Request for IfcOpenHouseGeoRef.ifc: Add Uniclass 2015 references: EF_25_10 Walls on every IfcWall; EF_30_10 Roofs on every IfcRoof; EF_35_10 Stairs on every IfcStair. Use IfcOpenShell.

First a look at what the model holds.

```python
import ifcopenshell

model = ifcopenshell.open("IfcOpenHouseGeoRef.ifc")
print(model.schema)
print("classifications:", [c.Name for c in model.by_type("IfcClassification")])
for ifc_class in ("IfcDoor", "IfcRoof", "IfcStair", "IfcWall", "IfcWindow"):
    print(ifc_class, len(model.by_type(ifc_class)))
```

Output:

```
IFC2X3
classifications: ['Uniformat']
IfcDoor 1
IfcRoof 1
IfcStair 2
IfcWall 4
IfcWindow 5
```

```python
import ifcopenshell
import ifcopenshell.api.classification

model = ifcopenshell.open("IfcOpenHouseGeoRef.ifc")

# IFC2X3 requires Source and Edition and has no link from the project to the system.
system = model.create_entity("IfcClassification", Source="NBS", Edition="2015", Name="Uniclass 2015")

codes = {
    "IfcWall": ("EF_25_10", "Walls"),
    "IfcRoof": ("EF_30_10", "Roofs"),
    "IfcStair": ("EF_35_10", "Stairs"),
}
for ifc_class, (code, name) in codes.items():
    products = model.by_type(ifc_class)
    ifcopenshell.api.classification.add_reference(
        model, products=products, classification=system, identification=code, name=name
    )
    print(code, len(products))

model.write("IfcOpenHouseGeoRef-out.ifc")
```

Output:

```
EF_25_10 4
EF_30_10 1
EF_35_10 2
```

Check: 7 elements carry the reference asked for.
